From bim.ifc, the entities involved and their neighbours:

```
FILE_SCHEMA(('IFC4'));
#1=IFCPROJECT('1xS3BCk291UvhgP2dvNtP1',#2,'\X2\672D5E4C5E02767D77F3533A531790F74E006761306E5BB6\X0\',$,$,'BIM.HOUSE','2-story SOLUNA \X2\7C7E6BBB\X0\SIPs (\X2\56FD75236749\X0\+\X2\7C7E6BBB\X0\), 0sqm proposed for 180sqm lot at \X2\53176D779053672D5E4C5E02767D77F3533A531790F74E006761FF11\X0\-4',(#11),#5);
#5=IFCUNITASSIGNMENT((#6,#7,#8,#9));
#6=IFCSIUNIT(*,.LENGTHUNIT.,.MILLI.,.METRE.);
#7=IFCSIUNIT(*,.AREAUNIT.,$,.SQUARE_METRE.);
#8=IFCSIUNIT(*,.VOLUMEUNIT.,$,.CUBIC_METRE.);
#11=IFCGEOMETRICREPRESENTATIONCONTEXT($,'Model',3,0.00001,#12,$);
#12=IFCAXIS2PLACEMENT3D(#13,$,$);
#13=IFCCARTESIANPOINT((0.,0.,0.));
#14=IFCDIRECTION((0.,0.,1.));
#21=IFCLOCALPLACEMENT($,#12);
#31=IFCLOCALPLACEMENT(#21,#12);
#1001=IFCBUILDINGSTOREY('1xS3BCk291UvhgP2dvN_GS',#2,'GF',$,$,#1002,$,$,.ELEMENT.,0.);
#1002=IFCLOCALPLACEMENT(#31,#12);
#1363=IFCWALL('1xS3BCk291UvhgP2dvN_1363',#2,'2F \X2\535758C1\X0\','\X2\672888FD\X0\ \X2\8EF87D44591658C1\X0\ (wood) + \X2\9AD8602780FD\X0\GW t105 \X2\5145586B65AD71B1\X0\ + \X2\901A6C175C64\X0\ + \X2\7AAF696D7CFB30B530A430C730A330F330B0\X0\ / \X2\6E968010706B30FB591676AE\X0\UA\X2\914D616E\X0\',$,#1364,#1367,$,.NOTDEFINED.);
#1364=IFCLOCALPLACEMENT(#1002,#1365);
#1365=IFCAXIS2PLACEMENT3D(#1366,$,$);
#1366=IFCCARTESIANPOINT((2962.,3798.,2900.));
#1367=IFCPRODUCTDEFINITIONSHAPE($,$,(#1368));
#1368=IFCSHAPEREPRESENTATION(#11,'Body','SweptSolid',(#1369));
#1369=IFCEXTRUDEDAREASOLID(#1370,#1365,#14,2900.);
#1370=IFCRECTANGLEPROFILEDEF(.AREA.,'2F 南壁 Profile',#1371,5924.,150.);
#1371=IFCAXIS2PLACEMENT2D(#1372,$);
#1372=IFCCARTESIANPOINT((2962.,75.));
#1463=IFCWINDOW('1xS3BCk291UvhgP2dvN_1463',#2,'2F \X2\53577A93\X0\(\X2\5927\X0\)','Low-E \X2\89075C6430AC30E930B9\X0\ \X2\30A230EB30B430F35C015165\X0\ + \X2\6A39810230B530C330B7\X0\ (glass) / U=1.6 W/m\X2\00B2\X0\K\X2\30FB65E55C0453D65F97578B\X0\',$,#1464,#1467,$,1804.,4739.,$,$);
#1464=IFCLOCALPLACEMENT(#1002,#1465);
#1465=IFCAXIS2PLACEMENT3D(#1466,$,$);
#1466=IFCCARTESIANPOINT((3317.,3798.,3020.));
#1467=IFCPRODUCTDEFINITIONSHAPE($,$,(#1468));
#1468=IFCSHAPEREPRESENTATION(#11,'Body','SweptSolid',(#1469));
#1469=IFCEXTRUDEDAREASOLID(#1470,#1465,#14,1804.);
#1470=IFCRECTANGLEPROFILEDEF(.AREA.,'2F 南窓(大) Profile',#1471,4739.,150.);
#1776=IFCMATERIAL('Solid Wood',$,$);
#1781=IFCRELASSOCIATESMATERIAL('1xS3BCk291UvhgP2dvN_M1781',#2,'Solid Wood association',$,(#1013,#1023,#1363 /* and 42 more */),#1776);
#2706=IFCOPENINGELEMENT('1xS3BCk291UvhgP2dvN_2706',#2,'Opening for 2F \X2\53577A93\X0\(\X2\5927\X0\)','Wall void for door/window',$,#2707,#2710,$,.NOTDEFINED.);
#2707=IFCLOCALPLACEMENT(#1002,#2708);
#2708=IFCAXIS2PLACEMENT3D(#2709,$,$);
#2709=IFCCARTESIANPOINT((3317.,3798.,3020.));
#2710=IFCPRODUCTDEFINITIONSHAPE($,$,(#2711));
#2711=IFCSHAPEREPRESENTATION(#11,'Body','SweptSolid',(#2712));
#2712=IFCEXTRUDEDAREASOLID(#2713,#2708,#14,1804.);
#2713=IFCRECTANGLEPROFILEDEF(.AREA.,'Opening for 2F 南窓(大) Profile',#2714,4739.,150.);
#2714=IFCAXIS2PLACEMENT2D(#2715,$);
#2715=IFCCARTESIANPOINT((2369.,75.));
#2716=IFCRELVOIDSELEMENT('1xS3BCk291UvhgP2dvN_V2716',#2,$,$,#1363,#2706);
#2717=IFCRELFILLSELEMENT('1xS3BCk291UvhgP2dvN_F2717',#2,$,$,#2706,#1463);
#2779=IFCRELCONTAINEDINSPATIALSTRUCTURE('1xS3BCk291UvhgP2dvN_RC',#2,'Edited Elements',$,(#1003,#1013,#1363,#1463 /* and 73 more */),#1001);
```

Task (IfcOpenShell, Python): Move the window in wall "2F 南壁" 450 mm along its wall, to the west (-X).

```python
import ifcopenshell
import ifcopenshell.api.geometry
import ifcopenshell.util.placement
import ifcopenshell.util.unit

model = ifcopenshell.open("bim.ifc")
unit_scale = ifcopenshell.util.unit.calculate_unit_scale(model)

window = model.by_guid("1xS3BCk291UvhgP2dvN_1463")
opening = window.FillsVoids[0].RelatingOpeningElement
wall = opening.VoidsElements[0].RelatingBuildingElement

wall_matrix = ifcopenshell.util.placement.get_local_placement(wall.ObjectPlacement)
shift = wall_matrix[:3, 0] * -0.45 / unit_scale
before = ifcopenshell.util.placement.get_local_placement(window.ObjectPlacement)[:3, 3].copy()

# The window is not placed relative to its opening, so move both.
for product in (opening, window):
    matrix = ifcopenshell.util.placement.get_local_placement(product.ObjectPlacement)
    matrix[:3, 3] += shift
    ifcopenshell.api.geometry.edit_object_placement(model, product=product, matrix=matrix, is_si=False)

after = ifcopenshell.util.placement.get_local_placement(window.ObjectPlacement)[:3, 3]
print("window moved by", (after - before).round(3) + 0.0)

model.write("bim_updated.ifc")
```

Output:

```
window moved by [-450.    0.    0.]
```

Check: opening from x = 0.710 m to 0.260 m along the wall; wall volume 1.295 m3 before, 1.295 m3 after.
